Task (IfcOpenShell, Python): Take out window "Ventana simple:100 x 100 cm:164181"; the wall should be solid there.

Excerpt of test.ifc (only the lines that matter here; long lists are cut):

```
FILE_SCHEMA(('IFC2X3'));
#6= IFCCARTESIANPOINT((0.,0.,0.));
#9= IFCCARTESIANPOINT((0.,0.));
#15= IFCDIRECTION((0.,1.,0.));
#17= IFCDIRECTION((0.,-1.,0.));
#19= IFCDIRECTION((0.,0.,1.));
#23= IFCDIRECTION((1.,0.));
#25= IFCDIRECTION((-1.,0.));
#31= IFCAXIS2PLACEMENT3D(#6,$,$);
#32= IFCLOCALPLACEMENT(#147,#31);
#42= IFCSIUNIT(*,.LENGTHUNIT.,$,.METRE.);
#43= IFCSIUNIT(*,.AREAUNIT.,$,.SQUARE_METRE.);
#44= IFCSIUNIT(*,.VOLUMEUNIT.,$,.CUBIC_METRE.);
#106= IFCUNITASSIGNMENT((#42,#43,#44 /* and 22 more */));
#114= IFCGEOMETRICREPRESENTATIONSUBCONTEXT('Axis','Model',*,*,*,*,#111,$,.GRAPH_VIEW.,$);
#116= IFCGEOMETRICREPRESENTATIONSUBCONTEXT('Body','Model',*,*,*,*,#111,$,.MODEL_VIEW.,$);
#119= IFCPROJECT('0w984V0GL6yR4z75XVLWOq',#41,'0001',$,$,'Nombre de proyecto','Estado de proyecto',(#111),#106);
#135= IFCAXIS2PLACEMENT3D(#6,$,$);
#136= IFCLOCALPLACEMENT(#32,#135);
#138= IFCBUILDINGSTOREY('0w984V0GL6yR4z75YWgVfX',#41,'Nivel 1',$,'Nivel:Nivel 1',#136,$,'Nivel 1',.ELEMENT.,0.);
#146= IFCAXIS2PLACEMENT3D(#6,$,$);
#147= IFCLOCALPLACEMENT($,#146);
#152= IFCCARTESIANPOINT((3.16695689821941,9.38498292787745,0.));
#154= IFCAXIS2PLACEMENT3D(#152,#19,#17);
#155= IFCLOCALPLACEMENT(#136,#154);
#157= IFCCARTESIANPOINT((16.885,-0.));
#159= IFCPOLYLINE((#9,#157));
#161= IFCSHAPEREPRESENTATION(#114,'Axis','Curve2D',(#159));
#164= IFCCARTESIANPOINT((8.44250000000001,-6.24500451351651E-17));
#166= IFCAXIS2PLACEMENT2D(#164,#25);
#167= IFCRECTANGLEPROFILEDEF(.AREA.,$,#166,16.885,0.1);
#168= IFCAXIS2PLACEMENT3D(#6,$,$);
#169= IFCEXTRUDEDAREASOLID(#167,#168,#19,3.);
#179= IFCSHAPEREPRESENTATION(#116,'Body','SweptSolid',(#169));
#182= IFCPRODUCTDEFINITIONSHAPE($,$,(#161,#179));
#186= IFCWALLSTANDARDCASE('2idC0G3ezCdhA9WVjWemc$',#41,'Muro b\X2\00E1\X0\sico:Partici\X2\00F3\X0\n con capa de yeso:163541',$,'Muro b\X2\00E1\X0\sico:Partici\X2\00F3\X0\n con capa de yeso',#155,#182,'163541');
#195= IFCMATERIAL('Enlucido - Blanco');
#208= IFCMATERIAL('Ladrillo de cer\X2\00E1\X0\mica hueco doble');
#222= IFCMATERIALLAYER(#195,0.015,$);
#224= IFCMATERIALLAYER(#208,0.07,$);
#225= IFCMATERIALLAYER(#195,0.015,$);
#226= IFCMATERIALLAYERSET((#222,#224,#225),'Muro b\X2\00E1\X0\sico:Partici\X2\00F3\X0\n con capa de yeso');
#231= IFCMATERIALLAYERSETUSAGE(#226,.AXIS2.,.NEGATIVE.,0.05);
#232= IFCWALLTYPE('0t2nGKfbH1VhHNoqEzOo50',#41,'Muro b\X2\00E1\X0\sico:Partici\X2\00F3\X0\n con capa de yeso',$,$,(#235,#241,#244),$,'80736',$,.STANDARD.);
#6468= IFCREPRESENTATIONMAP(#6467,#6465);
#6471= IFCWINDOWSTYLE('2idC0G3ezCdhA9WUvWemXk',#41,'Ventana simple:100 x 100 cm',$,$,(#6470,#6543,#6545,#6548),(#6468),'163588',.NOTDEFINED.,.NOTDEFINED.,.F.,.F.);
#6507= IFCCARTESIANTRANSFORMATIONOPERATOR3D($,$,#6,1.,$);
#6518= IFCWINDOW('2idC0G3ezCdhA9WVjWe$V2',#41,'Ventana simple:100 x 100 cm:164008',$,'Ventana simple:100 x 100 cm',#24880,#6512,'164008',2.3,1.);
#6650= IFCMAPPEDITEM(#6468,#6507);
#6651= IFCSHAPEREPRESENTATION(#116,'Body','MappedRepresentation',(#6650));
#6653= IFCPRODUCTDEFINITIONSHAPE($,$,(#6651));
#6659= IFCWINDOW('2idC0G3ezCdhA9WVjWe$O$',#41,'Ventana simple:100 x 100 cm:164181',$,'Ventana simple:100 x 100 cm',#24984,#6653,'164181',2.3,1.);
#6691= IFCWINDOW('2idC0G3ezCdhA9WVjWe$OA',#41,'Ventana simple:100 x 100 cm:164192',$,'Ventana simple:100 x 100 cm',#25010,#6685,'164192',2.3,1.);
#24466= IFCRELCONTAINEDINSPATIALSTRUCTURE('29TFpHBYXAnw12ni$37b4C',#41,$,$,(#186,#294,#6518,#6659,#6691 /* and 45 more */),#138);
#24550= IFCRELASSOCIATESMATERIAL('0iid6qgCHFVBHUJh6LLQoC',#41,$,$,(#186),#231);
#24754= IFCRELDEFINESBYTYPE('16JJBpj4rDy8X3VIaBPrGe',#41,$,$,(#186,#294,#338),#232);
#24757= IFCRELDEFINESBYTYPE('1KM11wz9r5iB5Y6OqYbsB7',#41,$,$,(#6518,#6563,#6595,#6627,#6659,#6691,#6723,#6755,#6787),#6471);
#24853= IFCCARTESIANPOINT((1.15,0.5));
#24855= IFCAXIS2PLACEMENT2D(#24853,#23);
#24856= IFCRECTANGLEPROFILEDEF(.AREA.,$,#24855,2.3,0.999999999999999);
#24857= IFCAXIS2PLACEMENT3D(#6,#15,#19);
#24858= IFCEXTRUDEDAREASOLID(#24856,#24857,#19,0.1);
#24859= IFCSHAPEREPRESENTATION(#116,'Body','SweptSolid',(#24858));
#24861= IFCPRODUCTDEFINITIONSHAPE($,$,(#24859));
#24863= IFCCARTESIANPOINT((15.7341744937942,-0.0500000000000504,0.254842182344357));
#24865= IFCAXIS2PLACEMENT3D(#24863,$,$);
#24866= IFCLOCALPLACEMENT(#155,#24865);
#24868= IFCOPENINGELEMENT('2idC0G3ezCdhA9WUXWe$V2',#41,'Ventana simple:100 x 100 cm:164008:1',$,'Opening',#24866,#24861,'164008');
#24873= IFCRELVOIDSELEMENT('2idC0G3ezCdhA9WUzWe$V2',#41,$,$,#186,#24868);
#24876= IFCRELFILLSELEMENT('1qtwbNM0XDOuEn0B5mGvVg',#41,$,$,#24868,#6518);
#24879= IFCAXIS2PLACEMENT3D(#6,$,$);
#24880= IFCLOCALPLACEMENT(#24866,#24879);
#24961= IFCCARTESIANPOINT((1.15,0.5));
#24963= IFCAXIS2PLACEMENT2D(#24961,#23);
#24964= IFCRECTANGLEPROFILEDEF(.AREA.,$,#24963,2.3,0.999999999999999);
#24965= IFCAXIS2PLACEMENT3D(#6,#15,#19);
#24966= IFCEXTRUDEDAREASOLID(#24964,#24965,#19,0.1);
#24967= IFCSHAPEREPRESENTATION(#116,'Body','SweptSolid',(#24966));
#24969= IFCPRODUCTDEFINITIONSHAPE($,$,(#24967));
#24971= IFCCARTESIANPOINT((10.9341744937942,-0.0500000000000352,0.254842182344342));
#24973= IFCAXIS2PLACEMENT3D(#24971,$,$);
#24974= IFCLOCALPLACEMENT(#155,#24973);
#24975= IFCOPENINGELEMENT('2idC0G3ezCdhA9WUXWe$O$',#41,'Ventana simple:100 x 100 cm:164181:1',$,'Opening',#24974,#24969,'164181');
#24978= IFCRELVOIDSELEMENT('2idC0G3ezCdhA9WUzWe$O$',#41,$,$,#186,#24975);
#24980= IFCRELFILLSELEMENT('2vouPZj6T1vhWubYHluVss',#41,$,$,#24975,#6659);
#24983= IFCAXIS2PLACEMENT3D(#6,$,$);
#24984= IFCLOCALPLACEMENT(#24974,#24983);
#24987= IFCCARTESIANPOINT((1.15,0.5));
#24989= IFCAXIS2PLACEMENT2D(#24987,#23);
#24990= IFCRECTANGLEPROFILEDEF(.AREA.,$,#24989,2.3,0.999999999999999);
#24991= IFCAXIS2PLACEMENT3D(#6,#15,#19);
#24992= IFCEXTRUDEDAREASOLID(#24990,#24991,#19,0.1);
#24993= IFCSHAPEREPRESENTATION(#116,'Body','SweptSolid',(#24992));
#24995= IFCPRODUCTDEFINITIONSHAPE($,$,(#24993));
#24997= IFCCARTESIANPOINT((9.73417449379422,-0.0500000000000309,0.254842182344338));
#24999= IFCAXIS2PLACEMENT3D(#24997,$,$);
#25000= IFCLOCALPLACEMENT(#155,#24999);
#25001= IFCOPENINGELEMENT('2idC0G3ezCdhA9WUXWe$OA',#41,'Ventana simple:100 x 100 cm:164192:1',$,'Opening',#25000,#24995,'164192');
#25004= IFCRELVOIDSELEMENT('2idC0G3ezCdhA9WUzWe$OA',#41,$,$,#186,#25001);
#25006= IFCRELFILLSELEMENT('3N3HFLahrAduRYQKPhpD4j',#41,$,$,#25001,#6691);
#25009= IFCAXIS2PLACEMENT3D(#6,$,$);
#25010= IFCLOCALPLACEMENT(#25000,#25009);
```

```python
import ifcopenshell
import ifcopenshell.api.feature
import ifcopenshell.api.root
import ifcopenshell.geom
import ifcopenshell.util.shape

model = ifcopenshell.open("test.ifc")
settings = ifcopenshell.geom.settings()


def volume(element):
    """Net volume in cubic metres, openings subtracted."""
    shape = ifcopenshell.geom.create_shape(settings, element)
    return ifcopenshell.util.shape.get_volume(shape.geometry)


window = model.by_id(6659)
opening = window.FillsVoids[0].RelatingOpeningElement
wall = opening.VoidsElements[0].RelatingBuildingElement
before = volume(wall)

ifcopenshell.api.root.remove_product(model, product=window)
ifcopenshell.api.feature.remove_feature(model, feature=opening)

after = volume(wall)

print(f"wall volume {before:.3f} -> {after:.3f} m3")

model.write("test_updated.ifc")
```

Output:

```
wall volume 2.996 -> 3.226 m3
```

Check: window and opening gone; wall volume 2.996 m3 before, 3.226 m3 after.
